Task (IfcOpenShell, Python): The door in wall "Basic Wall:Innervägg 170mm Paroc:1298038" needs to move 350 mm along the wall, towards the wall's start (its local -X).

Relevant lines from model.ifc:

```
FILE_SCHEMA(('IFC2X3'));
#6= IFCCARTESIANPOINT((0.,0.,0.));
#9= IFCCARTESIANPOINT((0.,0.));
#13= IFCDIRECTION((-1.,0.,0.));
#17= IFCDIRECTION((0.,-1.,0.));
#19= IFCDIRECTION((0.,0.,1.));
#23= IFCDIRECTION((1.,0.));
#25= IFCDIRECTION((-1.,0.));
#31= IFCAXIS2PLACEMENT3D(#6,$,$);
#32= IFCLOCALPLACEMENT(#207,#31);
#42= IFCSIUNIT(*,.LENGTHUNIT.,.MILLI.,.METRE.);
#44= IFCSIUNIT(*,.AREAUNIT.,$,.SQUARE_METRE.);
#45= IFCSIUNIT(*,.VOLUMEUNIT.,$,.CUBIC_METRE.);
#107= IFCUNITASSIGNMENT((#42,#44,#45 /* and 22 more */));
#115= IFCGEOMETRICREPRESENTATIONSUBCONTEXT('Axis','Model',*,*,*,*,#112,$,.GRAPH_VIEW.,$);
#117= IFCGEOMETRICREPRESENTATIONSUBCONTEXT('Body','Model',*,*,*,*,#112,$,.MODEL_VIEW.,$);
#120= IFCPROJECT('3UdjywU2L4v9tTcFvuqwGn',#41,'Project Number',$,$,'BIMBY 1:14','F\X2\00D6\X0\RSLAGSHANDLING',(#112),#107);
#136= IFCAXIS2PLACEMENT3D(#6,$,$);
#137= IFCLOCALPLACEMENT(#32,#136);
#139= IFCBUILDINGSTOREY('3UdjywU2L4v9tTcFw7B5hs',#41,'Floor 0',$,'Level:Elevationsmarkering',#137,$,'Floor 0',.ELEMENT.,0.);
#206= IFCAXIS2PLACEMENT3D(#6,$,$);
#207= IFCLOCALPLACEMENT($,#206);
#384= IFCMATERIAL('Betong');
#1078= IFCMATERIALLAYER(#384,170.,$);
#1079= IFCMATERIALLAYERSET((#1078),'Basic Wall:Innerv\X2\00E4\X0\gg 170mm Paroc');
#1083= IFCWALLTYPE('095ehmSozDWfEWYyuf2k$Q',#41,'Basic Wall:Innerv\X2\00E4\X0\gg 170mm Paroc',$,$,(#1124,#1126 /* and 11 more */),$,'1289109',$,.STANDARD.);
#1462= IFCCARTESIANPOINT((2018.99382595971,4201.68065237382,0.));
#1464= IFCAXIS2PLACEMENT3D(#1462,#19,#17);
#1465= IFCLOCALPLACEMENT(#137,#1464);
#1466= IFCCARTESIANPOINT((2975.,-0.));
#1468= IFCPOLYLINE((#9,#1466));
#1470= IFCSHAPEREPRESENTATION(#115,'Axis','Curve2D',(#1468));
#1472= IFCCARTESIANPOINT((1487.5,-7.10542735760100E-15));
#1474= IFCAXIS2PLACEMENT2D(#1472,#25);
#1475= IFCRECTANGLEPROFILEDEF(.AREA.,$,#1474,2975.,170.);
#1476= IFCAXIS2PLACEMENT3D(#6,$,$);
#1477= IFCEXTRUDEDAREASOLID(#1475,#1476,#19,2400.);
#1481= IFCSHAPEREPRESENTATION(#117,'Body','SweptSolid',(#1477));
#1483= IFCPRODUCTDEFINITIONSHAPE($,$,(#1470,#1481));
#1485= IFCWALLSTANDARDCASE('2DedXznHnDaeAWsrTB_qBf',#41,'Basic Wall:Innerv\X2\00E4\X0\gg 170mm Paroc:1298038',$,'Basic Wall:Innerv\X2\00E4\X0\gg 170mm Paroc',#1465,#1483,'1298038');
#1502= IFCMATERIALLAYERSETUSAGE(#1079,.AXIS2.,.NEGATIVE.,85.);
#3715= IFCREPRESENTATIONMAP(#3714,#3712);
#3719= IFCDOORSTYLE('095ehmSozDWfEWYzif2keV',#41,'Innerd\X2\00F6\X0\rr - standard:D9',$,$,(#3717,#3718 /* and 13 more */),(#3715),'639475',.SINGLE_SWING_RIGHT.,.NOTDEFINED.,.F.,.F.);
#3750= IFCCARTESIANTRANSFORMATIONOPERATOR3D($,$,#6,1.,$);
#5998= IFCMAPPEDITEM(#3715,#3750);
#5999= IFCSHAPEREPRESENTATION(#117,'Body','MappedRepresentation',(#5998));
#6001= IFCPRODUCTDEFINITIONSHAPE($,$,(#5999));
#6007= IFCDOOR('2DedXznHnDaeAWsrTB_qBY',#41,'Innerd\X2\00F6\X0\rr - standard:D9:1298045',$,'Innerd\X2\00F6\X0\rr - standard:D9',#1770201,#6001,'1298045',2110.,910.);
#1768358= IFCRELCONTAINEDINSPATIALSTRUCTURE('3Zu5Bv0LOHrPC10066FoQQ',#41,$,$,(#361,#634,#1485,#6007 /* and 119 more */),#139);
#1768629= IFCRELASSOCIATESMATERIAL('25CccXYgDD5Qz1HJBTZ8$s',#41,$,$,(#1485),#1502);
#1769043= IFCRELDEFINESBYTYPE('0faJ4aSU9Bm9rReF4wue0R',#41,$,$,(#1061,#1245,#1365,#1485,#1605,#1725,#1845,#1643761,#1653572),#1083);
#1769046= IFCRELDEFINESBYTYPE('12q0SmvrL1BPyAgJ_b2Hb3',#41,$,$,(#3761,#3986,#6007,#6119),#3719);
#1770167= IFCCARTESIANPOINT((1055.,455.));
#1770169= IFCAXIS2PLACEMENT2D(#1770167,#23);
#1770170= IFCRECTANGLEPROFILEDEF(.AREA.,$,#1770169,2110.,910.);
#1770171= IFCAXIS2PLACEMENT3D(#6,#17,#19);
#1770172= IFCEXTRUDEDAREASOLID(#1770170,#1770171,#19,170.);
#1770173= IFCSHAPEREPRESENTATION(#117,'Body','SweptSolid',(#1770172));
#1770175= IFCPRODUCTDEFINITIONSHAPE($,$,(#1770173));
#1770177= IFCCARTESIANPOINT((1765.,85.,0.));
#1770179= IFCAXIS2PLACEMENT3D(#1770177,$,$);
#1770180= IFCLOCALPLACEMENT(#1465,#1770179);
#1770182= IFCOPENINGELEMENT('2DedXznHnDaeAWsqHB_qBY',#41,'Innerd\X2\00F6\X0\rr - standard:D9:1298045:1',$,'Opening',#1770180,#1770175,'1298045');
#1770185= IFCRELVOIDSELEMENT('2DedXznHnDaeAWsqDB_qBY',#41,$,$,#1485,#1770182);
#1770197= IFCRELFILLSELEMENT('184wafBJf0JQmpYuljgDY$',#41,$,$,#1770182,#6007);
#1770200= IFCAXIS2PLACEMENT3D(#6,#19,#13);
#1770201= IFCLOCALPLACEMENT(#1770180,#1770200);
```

```python
import ifcopenshell
import ifcopenshell.api.geometry
import ifcopenshell.util.placement
import ifcopenshell.util.unit

model = ifcopenshell.open("model.ifc")
unit_scale = ifcopenshell.util.unit.calculate_unit_scale(model)

door = model.by_guid("2DedXznHnDaeAWsrTB_qBY")
opening = door.FillsVoids[0].RelatingOpeningElement
wall = opening.VoidsElements[0].RelatingBuildingElement

wall_matrix = ifcopenshell.util.placement.get_local_placement(wall.ObjectPlacement)
shift = wall_matrix[:3, 0] * -0.35 / unit_scale
before = ifcopenshell.util.placement.get_local_placement(door.ObjectPlacement)[:3, 3].copy()

# The door is placed relative to its opening, so it follows when the opening moves.
matrix = ifcopenshell.util.placement.get_local_placement(opening.ObjectPlacement)
matrix[:3, 3] += shift
ifcopenshell.api.geometry.edit_object_placement(
    model, product=opening, matrix=matrix, is_si=False, should_transform_children=True
)

after = ifcopenshell.util.placement.get_local_placement(door.ObjectPlacement)[:3, 3]
print("door moved by", (after - before).round(3) + 0.0)

model.write("model-out.ifc")
```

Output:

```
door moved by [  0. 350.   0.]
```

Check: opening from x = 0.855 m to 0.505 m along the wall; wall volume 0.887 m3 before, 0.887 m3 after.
